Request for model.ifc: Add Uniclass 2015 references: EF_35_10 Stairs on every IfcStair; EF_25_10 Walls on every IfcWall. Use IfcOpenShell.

First a look at what the model holds.

```python
import ifcopenshell

model = ifcopenshell.open("model.ifc")
print(model.schema)
print("classifications:", [c.Name for c in model.by_type("IfcClassification")])
for ifc_class in ("IfcDoor", "IfcRoof", "IfcStair", "IfcWall", "IfcWindow"):
    print(ifc_class, len(model.by_type(ifc_class)))
```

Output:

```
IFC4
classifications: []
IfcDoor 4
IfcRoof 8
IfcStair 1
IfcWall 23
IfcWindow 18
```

```python
import ifcopenshell
import ifcopenshell.api.classification

model = ifcopenshell.open("model.ifc")

system = ifcopenshell.api.classification.add_classification(model, classification="Uniclass 2015")

codes = {
    "IfcStair": ("EF_35_10", "Stairs"),
    "IfcWall": ("EF_25_10", "Walls"),
}
for ifc_class, (code, name) in codes.items():
    products = model.by_type(ifc_class)
    ifcopenshell.api.classification.add_reference(
        model, products=products, classification=system, identification=code, name=name
    )
    print(code, len(products))

model.write("model_v2.ifc")
```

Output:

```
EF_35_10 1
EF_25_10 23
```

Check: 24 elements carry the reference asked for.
